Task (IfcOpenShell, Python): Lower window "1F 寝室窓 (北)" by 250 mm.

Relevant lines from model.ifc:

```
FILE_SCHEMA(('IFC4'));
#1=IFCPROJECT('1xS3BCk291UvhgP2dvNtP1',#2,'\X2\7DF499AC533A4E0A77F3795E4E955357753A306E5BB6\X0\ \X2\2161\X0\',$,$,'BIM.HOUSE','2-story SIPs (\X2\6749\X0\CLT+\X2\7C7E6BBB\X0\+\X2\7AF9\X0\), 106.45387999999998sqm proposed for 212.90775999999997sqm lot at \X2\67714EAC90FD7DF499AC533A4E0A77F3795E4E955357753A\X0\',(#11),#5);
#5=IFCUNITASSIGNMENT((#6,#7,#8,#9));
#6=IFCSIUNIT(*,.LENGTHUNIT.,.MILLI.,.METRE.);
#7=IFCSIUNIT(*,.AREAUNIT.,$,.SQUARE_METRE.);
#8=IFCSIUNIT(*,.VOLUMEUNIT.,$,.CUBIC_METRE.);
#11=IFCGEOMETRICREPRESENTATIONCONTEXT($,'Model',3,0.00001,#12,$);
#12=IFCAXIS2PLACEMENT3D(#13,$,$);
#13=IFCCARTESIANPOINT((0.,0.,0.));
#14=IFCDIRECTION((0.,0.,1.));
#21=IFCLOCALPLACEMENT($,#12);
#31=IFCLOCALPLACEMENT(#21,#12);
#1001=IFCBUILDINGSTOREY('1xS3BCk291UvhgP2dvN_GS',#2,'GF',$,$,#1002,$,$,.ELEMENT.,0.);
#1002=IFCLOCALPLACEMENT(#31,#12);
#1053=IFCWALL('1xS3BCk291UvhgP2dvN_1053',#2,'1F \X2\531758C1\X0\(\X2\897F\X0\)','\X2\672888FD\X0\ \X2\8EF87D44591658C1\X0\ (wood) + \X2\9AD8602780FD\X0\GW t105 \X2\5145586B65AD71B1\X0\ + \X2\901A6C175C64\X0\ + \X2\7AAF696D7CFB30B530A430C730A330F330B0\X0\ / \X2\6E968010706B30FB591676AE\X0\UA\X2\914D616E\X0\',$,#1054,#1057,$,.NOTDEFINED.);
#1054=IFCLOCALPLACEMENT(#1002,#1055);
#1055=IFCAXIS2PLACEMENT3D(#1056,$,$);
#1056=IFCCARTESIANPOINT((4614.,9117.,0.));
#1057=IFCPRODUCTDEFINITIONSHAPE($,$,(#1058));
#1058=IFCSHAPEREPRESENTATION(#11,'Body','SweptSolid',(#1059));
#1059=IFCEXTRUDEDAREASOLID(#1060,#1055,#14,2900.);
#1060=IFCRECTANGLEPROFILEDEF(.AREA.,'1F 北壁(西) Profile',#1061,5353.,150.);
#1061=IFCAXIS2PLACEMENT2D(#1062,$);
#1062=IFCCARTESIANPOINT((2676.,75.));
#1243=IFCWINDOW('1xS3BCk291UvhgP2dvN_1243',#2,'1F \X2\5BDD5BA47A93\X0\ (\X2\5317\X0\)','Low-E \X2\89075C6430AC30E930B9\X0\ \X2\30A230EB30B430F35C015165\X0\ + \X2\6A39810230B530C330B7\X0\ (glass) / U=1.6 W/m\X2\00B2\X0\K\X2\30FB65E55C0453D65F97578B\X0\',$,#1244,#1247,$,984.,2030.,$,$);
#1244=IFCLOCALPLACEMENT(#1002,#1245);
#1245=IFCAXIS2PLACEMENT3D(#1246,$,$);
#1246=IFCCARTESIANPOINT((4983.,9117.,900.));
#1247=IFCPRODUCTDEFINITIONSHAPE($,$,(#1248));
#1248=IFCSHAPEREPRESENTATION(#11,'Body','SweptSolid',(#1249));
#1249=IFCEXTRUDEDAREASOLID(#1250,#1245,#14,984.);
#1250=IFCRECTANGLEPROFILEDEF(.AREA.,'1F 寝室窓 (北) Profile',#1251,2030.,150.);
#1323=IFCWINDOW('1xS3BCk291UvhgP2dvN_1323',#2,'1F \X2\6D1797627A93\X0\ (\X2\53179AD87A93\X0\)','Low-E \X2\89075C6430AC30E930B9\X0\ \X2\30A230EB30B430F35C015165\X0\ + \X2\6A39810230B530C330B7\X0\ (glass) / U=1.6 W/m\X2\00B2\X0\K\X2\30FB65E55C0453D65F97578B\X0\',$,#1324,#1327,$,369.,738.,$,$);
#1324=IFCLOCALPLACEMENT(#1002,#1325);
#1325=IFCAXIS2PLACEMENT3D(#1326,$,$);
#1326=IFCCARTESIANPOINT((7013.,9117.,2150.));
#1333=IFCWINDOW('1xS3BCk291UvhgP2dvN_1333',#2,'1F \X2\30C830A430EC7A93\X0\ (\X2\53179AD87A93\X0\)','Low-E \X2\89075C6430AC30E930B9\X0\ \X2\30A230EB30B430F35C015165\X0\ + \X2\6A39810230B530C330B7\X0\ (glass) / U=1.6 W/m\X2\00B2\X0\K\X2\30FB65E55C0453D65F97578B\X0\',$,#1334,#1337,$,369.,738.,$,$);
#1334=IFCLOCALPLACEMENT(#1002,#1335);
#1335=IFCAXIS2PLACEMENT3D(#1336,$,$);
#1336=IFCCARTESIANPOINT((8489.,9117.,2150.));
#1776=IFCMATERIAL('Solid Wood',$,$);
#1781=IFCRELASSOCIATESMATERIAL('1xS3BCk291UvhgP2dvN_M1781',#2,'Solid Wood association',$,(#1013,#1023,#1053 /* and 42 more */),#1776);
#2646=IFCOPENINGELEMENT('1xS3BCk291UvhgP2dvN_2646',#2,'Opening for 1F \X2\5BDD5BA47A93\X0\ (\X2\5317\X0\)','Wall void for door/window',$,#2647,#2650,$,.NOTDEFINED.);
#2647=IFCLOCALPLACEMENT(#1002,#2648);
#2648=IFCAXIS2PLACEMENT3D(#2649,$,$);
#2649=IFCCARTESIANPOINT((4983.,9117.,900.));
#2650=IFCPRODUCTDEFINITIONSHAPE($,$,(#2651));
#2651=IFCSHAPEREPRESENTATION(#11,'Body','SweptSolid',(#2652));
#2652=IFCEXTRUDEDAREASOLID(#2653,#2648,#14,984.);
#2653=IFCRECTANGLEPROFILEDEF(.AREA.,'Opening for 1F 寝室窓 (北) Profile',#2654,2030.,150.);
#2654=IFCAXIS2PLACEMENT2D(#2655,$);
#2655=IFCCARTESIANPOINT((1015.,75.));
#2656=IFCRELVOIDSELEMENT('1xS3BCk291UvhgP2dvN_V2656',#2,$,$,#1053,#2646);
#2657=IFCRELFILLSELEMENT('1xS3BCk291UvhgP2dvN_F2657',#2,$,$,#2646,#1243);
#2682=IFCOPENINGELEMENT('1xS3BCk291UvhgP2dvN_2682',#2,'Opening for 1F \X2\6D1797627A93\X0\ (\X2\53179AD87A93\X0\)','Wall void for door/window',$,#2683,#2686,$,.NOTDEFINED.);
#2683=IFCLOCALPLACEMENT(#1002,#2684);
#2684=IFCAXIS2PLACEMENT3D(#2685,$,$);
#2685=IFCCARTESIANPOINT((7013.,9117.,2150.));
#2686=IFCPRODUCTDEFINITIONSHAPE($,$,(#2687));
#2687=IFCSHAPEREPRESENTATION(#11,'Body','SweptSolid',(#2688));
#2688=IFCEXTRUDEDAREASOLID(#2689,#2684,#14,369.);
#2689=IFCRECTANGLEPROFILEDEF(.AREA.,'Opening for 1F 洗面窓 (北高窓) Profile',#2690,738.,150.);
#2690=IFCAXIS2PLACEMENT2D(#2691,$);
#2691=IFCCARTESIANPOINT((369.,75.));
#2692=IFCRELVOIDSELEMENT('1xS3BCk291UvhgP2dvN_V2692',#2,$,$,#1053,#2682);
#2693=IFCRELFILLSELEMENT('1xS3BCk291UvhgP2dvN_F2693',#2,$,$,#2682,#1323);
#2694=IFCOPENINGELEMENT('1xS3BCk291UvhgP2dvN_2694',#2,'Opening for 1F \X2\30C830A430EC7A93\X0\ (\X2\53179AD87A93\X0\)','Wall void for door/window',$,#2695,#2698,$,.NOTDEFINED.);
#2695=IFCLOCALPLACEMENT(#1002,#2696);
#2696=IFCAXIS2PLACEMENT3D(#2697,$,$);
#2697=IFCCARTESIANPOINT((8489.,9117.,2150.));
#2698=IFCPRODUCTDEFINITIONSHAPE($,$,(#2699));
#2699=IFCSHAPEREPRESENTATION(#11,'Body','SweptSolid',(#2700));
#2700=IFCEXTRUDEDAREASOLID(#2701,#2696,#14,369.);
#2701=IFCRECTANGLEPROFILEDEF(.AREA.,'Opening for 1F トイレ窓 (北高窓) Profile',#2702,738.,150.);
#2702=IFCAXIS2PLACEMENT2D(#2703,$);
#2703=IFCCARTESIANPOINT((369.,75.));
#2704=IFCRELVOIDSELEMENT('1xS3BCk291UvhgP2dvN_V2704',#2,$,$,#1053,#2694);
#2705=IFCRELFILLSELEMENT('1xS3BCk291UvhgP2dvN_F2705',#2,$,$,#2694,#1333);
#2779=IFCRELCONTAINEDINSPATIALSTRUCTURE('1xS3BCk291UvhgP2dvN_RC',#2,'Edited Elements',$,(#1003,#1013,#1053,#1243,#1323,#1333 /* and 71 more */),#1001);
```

```python
import numpy as np
import ifcopenshell
import ifcopenshell.api.geometry
import ifcopenshell.util.placement
import ifcopenshell.util.unit

model = ifcopenshell.open("model.ifc")
unit_scale = ifcopenshell.util.unit.calculate_unit_scale(model)

window = model.by_guid("1xS3BCk291UvhgP2dvN_1243")
opening = window.FillsVoids[0].RelatingOpeningElement
dz = -0.25 / unit_scale

shift = np.array([0.0, 0.0, dz])
# The window is not placed relative to its opening, so move both.
for product in (opening, window):
    matrix = ifcopenshell.util.placement.get_local_placement(product.ObjectPlacement)
    matrix[:3, 3] += shift
    ifcopenshell.api.geometry.edit_object_placement(model, product=product, matrix=matrix, is_si=False)

print(f"moved by {dz * unit_scale:+.3f} m")

model.write("model-out.ifc")
```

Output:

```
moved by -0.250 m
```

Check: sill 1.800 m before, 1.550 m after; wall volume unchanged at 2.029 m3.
